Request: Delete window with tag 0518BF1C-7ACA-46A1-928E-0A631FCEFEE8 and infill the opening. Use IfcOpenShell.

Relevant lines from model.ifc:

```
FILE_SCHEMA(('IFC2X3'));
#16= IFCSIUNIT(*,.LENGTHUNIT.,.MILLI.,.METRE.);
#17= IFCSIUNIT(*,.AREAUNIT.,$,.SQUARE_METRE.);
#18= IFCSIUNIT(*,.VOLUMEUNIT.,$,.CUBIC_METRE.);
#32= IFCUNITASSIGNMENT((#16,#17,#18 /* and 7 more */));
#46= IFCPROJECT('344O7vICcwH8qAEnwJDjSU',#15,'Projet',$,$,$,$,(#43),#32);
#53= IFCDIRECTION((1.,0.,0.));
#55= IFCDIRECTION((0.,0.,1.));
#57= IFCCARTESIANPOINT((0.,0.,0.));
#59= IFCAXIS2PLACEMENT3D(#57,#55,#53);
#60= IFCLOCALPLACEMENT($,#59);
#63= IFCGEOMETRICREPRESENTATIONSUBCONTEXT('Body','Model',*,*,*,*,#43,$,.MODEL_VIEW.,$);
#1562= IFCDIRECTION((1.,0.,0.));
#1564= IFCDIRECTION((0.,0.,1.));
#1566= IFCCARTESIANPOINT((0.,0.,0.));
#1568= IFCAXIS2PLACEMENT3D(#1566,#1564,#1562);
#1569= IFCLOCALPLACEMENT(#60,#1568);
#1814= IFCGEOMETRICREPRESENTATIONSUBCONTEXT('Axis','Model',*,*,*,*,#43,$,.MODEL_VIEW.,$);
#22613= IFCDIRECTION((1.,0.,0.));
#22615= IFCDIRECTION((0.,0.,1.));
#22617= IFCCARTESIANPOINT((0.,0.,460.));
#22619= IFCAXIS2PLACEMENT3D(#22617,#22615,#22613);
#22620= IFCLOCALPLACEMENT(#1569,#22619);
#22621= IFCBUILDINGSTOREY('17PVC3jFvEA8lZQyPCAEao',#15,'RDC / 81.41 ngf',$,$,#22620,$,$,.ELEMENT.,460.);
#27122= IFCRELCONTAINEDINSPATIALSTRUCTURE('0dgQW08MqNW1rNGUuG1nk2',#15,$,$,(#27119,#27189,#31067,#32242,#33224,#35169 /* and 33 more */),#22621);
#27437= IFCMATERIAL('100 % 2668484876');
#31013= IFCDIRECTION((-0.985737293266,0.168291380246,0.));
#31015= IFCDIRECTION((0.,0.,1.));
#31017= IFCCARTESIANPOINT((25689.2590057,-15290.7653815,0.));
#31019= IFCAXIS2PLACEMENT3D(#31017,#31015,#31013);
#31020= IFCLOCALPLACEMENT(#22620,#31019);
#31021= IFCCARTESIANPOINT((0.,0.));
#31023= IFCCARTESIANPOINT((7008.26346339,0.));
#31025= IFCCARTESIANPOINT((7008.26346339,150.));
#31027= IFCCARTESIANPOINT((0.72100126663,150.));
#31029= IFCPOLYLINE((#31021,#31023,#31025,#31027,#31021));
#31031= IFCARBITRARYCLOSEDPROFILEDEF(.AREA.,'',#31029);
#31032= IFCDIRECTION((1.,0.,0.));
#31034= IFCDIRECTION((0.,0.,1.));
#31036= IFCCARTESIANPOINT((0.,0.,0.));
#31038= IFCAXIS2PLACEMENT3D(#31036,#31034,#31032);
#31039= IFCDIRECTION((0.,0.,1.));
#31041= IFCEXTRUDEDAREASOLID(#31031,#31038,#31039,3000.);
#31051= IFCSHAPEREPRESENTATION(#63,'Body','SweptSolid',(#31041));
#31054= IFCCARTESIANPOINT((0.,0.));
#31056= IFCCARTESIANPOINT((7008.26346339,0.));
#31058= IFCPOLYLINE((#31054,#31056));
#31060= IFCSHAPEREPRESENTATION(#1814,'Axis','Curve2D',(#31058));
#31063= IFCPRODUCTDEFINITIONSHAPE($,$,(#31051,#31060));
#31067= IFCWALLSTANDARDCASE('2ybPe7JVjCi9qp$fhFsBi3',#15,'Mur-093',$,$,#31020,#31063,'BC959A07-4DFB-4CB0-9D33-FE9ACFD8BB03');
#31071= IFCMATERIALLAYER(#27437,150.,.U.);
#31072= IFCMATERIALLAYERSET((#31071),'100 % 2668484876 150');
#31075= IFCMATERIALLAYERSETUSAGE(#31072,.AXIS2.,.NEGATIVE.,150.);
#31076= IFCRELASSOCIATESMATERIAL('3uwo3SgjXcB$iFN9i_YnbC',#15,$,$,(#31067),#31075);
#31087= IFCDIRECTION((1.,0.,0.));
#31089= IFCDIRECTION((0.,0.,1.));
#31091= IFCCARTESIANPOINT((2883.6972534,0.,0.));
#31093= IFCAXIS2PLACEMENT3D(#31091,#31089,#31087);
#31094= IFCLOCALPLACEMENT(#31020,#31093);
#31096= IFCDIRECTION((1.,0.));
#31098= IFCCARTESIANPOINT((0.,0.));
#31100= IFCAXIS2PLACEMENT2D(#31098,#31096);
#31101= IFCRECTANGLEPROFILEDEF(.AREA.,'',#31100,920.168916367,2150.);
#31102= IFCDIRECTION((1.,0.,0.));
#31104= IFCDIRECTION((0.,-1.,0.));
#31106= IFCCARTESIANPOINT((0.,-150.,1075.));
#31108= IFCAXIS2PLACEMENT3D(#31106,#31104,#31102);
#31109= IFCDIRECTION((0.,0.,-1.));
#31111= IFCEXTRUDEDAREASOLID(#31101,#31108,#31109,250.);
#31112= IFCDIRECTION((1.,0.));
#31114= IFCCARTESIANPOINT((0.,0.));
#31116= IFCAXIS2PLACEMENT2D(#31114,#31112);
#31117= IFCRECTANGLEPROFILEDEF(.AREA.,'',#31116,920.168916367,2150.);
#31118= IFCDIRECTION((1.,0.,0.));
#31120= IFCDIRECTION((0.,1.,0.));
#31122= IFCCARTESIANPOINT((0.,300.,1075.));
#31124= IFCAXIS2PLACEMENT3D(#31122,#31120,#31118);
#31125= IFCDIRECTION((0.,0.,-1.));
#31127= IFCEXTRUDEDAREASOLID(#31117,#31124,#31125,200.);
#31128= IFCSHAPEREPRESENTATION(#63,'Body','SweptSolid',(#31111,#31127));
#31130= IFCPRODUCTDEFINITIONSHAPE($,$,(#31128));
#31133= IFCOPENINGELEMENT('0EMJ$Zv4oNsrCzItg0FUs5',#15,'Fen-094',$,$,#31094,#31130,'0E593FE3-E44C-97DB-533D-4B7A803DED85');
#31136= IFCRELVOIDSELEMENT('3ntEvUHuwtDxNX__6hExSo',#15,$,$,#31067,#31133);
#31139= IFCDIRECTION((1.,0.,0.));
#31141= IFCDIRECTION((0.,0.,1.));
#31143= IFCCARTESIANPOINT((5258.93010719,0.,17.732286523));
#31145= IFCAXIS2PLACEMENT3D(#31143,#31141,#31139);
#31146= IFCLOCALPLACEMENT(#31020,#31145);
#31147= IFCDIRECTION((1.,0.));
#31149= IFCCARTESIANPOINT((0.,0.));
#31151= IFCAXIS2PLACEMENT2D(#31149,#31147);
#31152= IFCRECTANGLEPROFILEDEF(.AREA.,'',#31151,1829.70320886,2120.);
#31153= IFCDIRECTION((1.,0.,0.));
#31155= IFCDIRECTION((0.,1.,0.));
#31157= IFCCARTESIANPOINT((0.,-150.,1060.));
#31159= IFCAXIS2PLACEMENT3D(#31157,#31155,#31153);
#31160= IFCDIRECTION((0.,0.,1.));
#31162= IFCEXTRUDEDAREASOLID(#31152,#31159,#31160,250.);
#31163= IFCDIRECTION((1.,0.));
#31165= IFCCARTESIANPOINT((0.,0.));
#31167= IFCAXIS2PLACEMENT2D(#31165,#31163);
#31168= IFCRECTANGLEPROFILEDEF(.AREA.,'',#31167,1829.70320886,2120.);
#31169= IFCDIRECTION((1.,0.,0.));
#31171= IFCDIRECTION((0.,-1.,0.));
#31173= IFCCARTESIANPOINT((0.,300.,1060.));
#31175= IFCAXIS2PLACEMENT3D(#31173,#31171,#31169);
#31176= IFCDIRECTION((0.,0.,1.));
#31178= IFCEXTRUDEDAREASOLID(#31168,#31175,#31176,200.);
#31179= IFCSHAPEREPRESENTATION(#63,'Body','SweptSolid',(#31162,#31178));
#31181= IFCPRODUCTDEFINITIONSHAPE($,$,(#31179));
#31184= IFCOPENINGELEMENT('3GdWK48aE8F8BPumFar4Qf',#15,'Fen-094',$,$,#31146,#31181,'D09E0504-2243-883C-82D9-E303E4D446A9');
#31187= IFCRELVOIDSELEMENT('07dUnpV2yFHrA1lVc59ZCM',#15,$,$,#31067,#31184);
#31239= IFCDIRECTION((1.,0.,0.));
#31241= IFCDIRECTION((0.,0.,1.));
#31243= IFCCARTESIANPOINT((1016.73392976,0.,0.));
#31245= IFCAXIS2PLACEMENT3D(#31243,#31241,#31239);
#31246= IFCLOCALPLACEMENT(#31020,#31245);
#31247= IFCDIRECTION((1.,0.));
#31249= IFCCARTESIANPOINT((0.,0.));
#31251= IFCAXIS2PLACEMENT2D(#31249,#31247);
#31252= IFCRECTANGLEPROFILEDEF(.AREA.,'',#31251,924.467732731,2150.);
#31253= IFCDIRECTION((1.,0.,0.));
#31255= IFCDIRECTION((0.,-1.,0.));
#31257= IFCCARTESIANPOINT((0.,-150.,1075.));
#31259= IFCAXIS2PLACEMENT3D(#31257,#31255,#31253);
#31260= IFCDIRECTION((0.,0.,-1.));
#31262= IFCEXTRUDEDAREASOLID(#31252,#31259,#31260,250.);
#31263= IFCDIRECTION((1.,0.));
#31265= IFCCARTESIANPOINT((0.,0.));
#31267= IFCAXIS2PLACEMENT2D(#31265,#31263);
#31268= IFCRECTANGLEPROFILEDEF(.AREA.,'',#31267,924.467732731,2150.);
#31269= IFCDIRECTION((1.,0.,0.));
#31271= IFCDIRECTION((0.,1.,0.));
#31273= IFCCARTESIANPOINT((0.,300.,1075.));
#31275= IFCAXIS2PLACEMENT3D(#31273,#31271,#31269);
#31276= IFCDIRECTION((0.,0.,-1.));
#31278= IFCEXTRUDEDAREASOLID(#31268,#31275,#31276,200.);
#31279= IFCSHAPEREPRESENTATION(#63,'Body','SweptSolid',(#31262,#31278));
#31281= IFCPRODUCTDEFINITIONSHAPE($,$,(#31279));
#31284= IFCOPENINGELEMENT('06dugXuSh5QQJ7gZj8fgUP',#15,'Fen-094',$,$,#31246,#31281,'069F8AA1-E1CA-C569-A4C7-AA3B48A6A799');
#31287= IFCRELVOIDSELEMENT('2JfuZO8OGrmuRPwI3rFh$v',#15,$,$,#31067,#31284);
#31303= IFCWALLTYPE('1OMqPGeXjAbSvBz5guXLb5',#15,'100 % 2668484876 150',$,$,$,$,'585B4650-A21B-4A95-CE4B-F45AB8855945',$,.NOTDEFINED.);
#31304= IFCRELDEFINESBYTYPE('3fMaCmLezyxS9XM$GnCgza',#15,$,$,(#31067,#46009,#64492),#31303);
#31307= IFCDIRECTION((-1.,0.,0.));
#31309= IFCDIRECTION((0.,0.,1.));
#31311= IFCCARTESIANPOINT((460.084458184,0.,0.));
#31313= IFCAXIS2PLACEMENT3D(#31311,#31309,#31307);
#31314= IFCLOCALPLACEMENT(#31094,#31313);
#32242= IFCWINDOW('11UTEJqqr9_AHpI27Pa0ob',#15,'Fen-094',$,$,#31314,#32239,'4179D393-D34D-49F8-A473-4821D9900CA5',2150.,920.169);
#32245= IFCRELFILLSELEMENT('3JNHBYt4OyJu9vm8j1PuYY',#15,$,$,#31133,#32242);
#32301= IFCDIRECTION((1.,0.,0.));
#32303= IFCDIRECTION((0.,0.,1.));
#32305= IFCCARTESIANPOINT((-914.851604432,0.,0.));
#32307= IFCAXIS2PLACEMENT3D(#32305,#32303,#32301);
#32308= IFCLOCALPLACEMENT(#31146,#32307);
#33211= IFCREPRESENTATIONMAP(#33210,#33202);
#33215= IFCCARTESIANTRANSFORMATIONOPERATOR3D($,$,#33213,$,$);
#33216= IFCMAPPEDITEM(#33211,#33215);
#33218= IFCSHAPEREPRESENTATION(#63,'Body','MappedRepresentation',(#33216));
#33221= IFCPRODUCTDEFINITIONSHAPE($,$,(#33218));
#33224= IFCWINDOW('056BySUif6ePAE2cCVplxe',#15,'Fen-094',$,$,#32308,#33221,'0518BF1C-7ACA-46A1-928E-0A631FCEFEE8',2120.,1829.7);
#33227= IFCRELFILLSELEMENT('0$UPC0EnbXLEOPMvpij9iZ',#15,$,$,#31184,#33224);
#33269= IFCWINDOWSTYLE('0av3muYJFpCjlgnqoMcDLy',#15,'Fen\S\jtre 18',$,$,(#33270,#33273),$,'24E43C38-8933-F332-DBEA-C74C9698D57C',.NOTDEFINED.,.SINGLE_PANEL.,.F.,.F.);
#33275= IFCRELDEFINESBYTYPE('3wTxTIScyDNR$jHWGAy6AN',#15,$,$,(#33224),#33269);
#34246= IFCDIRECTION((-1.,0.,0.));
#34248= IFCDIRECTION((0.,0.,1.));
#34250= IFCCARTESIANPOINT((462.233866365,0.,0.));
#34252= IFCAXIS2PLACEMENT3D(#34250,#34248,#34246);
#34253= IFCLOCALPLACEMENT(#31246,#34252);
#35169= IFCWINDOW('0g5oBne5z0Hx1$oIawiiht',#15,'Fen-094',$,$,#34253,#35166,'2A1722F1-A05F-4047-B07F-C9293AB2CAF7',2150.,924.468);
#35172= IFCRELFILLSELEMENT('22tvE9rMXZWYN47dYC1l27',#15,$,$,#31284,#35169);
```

```python
import ifcopenshell
import ifcopenshell.api.feature
import ifcopenshell.api.root
import ifcopenshell.geom
import ifcopenshell.util.shape

model = ifcopenshell.open("model.ifc")
settings = ifcopenshell.geom.settings()


def volume(element):
    """Net volume in cubic metres, openings subtracted."""
    shape = ifcopenshell.geom.create_shape(settings, element)
    return ifcopenshell.util.shape.get_volume(shape.geometry)


window = model.by_guid("056BySUif6ePAE2cCVplxe")
opening = window.FillsVoids[0].RelatingOpeningElement
wall = opening.VoidsElements[0].RelatingBuildingElement
before = volume(wall)

ifcopenshell.api.root.remove_product(model, product=window)
ifcopenshell.api.feature.remove_feature(model, feature=opening)

after = volume(wall)

print(f"wall volume {before:.3f} -> {after:.3f} m3")

model.write("model_edited.ifc")
```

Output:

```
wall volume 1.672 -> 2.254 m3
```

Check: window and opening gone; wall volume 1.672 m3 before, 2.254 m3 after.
